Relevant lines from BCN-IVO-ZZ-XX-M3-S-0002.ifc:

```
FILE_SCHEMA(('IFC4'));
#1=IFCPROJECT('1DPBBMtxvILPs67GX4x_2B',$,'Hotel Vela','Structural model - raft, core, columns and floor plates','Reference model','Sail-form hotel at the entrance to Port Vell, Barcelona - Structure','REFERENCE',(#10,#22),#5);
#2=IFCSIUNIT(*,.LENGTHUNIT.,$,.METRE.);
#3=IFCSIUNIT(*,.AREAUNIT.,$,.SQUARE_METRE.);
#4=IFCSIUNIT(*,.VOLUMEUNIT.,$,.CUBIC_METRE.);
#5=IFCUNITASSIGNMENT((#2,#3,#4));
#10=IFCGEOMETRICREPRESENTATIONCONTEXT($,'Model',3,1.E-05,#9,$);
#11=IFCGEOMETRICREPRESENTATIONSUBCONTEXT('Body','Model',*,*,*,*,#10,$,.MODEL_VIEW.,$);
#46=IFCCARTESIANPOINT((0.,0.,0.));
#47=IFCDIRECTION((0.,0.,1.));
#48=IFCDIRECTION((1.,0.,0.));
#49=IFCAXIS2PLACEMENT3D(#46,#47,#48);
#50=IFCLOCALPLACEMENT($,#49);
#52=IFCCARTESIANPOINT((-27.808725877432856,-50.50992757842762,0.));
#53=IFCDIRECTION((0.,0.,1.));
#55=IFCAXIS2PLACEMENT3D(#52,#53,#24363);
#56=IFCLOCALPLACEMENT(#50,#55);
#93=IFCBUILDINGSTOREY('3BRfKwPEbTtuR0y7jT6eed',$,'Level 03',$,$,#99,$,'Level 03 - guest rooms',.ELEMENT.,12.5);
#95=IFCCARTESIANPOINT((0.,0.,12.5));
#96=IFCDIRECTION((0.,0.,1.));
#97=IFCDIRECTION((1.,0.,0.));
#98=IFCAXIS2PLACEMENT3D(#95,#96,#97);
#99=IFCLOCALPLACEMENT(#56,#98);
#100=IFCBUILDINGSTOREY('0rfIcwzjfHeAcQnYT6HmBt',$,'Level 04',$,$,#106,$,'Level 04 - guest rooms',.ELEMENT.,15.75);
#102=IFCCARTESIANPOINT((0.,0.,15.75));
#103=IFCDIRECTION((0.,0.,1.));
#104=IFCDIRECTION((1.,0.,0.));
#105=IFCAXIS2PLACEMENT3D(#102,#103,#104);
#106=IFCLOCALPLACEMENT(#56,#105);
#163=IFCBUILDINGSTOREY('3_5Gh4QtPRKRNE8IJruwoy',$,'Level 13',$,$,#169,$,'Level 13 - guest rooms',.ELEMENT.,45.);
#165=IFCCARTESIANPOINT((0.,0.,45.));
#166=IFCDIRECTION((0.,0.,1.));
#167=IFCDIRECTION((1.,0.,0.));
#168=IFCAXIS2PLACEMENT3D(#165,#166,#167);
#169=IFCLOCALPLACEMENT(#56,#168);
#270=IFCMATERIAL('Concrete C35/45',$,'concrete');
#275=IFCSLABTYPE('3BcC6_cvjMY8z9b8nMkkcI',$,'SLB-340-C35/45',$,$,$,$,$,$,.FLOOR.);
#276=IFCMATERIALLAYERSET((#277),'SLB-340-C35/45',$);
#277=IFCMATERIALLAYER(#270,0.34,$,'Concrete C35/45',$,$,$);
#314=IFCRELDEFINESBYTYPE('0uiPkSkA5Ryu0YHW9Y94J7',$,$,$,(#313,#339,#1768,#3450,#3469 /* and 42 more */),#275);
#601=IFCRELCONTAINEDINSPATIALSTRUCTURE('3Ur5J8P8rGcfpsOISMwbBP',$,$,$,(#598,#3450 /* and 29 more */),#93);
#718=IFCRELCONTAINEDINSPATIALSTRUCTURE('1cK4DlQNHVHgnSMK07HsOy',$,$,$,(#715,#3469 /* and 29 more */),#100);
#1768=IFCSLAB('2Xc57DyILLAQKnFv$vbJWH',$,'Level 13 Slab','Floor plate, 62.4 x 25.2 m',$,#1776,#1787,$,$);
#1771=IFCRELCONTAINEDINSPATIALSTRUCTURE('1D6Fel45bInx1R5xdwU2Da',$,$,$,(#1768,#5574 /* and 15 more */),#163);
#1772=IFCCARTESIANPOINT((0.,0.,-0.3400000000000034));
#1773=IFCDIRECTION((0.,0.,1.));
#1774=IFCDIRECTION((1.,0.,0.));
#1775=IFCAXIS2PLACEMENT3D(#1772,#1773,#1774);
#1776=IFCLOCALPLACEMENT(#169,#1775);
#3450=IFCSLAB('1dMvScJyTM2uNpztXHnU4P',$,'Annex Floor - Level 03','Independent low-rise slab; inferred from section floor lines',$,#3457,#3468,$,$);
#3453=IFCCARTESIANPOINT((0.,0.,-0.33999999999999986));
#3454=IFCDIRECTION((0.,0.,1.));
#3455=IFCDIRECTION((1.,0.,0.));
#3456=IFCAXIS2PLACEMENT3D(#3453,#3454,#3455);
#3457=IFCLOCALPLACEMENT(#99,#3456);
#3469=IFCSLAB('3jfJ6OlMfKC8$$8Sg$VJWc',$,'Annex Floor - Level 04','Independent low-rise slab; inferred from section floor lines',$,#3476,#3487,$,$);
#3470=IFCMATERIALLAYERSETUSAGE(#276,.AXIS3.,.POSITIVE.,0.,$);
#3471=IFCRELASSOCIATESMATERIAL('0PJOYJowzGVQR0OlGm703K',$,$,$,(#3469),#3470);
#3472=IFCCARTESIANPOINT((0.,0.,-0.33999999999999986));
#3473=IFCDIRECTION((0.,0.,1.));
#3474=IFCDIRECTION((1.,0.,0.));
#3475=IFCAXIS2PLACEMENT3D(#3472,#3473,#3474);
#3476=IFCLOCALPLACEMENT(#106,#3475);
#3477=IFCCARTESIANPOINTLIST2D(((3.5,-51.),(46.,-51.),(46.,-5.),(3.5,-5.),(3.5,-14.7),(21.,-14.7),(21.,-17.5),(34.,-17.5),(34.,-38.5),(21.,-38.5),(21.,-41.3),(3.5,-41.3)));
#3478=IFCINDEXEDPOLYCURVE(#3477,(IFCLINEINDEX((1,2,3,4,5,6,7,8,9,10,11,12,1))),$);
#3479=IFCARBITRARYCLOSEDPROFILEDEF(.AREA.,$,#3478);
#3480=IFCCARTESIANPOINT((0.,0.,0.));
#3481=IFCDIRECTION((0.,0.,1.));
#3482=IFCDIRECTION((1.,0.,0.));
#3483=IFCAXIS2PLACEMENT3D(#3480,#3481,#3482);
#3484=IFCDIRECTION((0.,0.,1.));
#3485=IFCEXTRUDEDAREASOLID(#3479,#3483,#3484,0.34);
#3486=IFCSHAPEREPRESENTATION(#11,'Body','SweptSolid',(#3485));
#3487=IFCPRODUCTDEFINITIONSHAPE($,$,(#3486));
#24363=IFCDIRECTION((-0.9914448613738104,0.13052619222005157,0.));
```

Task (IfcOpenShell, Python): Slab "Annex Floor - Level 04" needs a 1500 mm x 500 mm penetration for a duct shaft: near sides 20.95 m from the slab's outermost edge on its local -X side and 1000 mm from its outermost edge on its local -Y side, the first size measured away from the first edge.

```python
import numpy as np
import ifcopenshell
import ifcopenshell.api.feature
import ifcopenshell.api.geometry
import ifcopenshell.api.root
import ifcopenshell.geom
import ifcopenshell.util.placement
import ifcopenshell.util.representation
import ifcopenshell.util.shape
import ifcopenshell.util.unit

model = ifcopenshell.open("BCN-IVO-ZZ-XX-M3-S-0002.ifc")
unit_scale = ifcopenshell.util.unit.calculate_unit_scale(model)
settings = ifcopenshell.geom.settings()


def volume(element):
    """Net volume in cubic metres, openings subtracted."""
    shape = ifcopenshell.geom.create_shape(settings, element)
    return ifcopenshell.util.shape.get_volume(shape.geometry)


slab = model.by_guid("3jfJ6OlMfKC8$$8Sg$VJWc")
before = volume(slab)

# Extent in the slab's own axes, in metres. The edges named are its -X and -Y sides.
slab_shape = ifcopenshell.geom.create_shape(settings, slab)
vertices = ifcopenshell.util.shape.get_vertices(slab_shape.geometry)
x_min, y_min, bottom = vertices.min(axis=0)
top = vertices[:, 2].max()

opening = ifcopenshell.api.root.create_entity(model, ifc_class="IfcOpeningElement", name="Duct shaft opening", predefined_type="OPENING")
context = ifcopenshell.util.representation.get_context(model, "Model", "Body", "MODEL_VIEW")
width, depth = 1.5, 0.5
outline = [(0.0, 0.0), (width, 0.0), (width, depth), (0.0, depth), (0.0, 0.0)]
# Overshoot both faces by 50 mm so the cut is clean.
shape = ifcopenshell.api.geometry.add_slab_representation(
    model, context=context, depth=top - bottom + 0.1, polyline=outline
)
ifcopenshell.api.geometry.assign_representation(model, product=opening, representation=shape)

matrix = ifcopenshell.util.placement.get_local_placement(slab.ObjectPlacement)
matrix[:, 3] = matrix @ np.append(np.array([x_min + 20.95, y_min + 1, bottom - 0.05]) / unit_scale, 1.0)
ifcopenshell.api.geometry.edit_object_placement(model, product=opening, matrix=matrix, is_si=False)
ifcopenshell.api.feature.add_feature(model, feature=opening, element=slab)

after = volume(slab)

print(f"slab volume {before:.3f} -> {after:.3f} m3")

model.write("BCN-IVO-ZZ-XX-M3-S-0002_v2.ifc")
```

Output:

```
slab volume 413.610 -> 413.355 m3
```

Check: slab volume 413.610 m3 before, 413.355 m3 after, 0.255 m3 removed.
